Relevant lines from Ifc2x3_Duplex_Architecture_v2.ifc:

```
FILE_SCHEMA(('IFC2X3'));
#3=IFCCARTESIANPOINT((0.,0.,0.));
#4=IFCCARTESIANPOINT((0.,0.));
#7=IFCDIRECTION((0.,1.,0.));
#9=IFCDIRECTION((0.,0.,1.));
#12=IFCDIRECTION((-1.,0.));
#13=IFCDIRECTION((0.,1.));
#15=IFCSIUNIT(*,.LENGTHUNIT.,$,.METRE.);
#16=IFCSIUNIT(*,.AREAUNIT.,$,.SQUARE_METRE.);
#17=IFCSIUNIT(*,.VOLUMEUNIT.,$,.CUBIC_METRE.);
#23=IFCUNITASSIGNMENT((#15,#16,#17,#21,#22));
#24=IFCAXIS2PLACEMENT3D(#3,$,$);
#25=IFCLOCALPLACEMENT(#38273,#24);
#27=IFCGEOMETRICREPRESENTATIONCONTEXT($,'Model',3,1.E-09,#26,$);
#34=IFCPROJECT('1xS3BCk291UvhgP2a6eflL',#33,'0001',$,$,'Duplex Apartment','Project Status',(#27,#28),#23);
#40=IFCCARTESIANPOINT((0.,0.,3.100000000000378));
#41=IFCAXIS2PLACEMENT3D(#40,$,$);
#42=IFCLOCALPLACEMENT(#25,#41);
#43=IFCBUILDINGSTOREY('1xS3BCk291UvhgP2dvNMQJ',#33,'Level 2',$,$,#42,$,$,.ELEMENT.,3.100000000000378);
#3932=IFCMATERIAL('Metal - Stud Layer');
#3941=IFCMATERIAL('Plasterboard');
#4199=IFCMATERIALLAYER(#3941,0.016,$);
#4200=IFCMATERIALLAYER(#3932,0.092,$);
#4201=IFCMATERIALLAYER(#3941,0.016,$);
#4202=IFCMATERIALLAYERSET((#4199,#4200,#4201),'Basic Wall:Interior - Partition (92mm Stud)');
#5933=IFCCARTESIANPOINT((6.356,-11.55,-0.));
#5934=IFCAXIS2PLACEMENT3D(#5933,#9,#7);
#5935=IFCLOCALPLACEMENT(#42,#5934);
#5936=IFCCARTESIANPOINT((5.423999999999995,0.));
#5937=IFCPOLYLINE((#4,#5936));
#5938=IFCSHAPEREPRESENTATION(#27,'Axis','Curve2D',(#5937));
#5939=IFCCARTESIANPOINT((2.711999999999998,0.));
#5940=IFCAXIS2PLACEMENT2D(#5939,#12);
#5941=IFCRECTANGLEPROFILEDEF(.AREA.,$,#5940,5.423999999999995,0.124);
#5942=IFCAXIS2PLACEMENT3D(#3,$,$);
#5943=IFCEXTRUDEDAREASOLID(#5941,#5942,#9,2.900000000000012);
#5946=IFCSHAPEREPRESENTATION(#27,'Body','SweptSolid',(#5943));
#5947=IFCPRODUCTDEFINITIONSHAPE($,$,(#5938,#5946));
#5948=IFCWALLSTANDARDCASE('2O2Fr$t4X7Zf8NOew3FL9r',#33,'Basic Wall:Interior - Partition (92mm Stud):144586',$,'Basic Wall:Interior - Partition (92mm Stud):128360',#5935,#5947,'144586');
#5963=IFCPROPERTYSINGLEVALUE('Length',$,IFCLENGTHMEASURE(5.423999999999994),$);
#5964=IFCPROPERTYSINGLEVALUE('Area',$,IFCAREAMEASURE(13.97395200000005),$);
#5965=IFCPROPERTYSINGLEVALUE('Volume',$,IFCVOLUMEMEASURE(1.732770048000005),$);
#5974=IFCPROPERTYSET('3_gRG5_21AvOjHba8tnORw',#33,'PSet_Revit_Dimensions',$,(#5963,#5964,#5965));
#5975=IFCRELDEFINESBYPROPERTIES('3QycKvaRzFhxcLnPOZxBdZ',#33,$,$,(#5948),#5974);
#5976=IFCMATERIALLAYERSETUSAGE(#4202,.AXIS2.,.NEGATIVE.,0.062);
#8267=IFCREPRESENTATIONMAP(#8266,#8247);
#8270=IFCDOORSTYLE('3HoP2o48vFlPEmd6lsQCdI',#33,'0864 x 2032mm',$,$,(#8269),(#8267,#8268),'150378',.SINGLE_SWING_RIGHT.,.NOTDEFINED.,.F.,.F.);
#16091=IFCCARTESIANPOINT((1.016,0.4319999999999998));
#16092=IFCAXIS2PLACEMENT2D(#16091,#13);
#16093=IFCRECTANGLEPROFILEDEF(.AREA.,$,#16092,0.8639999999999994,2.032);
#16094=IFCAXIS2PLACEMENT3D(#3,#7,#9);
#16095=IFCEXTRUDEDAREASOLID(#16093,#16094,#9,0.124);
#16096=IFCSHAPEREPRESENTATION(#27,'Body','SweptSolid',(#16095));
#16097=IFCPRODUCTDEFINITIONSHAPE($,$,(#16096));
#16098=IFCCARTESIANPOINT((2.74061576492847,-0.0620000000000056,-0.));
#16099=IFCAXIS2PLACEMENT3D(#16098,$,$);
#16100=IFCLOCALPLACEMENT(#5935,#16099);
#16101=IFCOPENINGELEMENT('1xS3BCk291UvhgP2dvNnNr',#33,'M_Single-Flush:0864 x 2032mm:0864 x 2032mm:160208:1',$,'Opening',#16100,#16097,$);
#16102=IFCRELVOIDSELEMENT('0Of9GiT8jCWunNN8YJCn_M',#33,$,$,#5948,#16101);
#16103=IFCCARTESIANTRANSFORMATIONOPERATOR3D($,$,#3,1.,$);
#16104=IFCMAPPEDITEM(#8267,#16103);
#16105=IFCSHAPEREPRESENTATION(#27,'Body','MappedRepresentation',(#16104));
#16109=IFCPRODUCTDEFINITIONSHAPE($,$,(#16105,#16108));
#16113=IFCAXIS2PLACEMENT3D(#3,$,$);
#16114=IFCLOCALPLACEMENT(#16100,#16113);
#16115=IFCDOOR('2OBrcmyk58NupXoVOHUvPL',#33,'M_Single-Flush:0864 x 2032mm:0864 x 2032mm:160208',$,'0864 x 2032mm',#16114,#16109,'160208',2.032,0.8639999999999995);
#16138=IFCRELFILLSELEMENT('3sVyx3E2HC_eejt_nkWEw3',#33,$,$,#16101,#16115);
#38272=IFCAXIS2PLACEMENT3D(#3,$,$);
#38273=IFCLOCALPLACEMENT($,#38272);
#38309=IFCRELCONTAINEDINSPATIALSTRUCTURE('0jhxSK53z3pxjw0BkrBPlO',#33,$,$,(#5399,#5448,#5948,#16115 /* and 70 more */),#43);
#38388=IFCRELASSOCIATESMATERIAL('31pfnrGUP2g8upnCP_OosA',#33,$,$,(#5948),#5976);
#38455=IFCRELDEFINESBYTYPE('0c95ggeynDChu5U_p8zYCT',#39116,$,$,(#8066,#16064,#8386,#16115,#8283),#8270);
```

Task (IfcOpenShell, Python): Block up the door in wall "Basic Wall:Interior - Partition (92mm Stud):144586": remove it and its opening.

```python
import ifcopenshell
import ifcopenshell.api.feature
import ifcopenshell.api.pset
import ifcopenshell.api.root
import ifcopenshell.geom
import ifcopenshell.util.element
import ifcopenshell.util.shape
import ifcopenshell.util.unit

model = ifcopenshell.open("Ifc2x3_Duplex_Architecture_v2.ifc")
area_scale = ifcopenshell.util.unit.calculate_unit_scale(model, "AREAUNIT")
volume_scale = ifcopenshell.util.unit.calculate_unit_scale(model, "VOLUMEUNIT")
settings = ifcopenshell.geom.settings()


def volume(element):
    """Net volume in cubic metres, openings subtracted."""
    shape = ifcopenshell.geom.create_shape(settings, element)
    return ifcopenshell.util.shape.get_volume(shape.geometry)


door = model.by_guid("2OBrcmyk58NupXoVOHUvPL")
opening = door.FillsVoids[0].RelatingOpeningElement
wall = opening.VoidsElements[0].RelatingBuildingElement
before = volume(wall)

ifcopenshell.api.root.remove_product(model, product=door)
ifcopenshell.api.feature.remove_feature(model, feature=opening)

after = volume(wall)
thickness = 0.124  # wall thickness in metres

# Update the wall's stored quantities.
pset = model.by_id(ifcopenshell.util.element.get_pset(wall, "PSet_Revit_Dimensions", should_inherit=False)["id"])
ifcopenshell.api.pset.edit_pset(model, pset=pset, properties={
    "Area": model.create_entity("IfcAreaMeasure", after / thickness / area_scale),
    "Volume": model.create_entity("IfcVolumeMeasure", after / volume_scale),
})

print(f"wall volume {before:.3f} -> {after:.3f} m3")

model.write("Ifc2x3_Duplex_Architecture_v2_edited.ifc")
```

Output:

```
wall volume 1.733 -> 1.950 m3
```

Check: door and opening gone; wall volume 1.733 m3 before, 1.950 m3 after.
